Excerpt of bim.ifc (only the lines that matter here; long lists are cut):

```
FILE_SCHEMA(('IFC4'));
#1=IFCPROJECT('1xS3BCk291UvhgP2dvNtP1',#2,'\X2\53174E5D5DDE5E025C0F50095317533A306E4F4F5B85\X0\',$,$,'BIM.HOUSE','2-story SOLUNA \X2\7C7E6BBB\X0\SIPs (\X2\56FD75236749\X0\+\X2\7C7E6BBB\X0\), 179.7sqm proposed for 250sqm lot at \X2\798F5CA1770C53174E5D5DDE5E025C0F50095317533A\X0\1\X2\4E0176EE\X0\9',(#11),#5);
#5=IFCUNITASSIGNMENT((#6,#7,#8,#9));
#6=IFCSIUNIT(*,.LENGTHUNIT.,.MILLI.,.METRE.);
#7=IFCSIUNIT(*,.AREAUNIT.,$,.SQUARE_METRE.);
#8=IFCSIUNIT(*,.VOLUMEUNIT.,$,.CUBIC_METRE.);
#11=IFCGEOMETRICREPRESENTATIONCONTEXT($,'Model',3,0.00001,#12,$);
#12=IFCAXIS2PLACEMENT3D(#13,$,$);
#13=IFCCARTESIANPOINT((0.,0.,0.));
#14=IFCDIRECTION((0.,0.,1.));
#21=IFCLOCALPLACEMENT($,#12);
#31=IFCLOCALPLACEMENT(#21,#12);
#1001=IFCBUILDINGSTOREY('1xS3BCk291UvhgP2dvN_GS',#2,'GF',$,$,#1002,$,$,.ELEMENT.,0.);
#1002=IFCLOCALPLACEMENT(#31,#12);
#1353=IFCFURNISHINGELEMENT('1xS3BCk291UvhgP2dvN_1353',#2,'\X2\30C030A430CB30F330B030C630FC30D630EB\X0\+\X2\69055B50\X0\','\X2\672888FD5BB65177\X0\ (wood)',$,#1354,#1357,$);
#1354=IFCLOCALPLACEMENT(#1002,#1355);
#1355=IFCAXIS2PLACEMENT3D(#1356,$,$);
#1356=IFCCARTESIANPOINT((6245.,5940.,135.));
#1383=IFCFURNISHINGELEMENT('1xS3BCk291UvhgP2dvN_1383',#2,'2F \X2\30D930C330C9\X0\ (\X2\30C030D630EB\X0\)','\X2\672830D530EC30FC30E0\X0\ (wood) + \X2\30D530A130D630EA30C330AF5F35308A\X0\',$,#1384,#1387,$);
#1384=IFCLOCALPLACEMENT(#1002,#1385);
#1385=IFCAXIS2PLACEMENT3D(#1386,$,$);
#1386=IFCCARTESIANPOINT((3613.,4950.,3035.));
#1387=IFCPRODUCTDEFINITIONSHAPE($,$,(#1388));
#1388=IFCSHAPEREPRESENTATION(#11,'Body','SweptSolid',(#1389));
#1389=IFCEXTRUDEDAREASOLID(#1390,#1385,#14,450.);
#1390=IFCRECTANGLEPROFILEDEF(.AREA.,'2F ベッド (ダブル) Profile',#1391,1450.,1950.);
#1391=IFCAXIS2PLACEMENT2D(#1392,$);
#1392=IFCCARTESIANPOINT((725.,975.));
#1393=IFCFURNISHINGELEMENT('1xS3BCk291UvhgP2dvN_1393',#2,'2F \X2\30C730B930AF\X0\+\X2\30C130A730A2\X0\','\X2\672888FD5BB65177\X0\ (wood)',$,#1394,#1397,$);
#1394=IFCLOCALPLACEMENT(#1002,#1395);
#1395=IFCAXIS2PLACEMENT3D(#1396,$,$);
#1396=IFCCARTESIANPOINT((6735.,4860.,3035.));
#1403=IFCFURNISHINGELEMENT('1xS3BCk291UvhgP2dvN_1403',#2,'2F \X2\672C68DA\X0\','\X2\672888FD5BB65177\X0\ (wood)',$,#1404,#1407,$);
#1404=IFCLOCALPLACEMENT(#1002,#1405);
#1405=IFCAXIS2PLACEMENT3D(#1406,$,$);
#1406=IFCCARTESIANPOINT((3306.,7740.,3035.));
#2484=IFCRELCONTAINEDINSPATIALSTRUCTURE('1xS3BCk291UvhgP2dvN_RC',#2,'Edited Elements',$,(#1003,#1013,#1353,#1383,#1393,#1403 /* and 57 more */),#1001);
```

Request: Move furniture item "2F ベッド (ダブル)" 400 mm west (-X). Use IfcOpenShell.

```python
import ifcopenshell
import ifcopenshell.api.geometry
import ifcopenshell.util.placement
import ifcopenshell.util.unit

model = ifcopenshell.open("bim.ifc")
unit_scale = ifcopenshell.util.unit.calculate_unit_scale(model)

item = model.by_guid("1xS3BCk291UvhgP2dvN_1383")
matrix = ifcopenshell.util.placement.get_local_placement(item.ObjectPlacement)
matrix[0, 3] -= 0.4 / unit_scale
ifcopenshell.api.geometry.edit_object_placement(model, product=item, matrix=matrix, is_si=False)

print(ifcopenshell.util.placement.get_local_placement(item.ObjectPlacement).round(3) + 0.0)

model.write("bim-out.ifc")
```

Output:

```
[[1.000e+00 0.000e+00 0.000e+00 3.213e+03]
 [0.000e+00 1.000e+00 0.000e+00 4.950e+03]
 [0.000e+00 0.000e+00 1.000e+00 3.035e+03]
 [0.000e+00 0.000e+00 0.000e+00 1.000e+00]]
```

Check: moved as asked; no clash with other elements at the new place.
